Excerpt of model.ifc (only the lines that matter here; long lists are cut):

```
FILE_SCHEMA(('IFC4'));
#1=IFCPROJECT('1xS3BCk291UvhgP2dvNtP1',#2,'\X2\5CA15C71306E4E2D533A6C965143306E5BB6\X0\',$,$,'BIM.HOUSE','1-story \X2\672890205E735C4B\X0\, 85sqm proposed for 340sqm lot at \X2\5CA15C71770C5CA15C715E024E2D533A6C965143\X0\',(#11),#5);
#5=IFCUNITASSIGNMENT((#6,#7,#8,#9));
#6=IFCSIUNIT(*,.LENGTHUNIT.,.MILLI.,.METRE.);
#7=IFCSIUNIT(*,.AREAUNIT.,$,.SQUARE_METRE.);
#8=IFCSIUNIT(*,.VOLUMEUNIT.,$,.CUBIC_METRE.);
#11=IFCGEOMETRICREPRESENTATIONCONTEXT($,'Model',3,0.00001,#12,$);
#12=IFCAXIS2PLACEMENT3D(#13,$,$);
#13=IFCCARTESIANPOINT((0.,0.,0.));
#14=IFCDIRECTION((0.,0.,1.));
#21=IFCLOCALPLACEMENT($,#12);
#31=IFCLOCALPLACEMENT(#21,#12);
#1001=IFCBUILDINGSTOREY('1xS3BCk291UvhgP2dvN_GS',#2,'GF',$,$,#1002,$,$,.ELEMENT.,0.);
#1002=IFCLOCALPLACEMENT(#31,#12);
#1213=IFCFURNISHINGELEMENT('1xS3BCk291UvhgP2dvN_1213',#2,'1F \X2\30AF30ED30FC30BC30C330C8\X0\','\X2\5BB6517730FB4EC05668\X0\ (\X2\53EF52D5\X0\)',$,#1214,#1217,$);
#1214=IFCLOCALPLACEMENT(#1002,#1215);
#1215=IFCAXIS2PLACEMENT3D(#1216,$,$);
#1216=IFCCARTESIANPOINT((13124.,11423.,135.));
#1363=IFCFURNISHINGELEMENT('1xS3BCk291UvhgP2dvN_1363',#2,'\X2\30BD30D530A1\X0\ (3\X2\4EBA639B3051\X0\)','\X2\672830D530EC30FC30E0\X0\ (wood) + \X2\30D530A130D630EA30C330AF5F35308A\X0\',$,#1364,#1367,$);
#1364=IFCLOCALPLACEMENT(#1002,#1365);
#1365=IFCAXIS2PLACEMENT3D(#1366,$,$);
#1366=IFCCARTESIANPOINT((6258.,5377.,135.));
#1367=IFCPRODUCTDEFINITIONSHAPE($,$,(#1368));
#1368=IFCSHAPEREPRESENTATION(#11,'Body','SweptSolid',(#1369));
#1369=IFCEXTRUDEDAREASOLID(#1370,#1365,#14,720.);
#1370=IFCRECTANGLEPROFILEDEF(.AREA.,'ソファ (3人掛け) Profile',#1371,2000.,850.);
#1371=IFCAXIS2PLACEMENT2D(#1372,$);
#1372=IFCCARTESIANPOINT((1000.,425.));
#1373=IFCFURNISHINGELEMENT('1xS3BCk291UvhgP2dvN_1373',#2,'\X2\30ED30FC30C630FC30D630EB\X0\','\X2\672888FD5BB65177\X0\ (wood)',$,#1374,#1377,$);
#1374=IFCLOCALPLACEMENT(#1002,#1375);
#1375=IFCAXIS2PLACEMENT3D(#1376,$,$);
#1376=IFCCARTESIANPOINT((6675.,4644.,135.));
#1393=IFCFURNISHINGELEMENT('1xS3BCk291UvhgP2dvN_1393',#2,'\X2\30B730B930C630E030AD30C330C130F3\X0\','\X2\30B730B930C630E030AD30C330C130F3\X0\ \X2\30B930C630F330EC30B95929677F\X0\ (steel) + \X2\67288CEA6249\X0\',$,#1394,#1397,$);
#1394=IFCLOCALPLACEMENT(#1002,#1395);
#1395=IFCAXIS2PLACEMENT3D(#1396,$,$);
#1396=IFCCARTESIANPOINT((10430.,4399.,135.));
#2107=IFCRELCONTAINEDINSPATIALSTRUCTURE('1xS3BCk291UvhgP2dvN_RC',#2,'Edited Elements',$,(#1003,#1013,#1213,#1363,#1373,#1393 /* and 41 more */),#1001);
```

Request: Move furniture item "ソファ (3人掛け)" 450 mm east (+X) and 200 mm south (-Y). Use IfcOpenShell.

```python
import ifcopenshell
import ifcopenshell.api.geometry
import ifcopenshell.util.placement
import ifcopenshell.util.unit

model = ifcopenshell.open("model.ifc")
unit_scale = ifcopenshell.util.unit.calculate_unit_scale(model)

item = model.by_id(1363)
matrix = ifcopenshell.util.placement.get_local_placement(item.ObjectPlacement)
matrix[0, 3] += 0.45 / unit_scale
matrix[1, 3] -= 0.2 / unit_scale
ifcopenshell.api.geometry.edit_object_placement(model, product=item, matrix=matrix, is_si=False)

print(ifcopenshell.util.placement.get_local_placement(item.ObjectPlacement).round(3) + 0.0)

model.write("model-out.ifc")
```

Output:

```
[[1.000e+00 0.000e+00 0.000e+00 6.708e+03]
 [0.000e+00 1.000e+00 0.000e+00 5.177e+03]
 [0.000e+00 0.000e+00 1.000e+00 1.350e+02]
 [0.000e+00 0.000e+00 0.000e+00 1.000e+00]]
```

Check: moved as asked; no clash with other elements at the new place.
